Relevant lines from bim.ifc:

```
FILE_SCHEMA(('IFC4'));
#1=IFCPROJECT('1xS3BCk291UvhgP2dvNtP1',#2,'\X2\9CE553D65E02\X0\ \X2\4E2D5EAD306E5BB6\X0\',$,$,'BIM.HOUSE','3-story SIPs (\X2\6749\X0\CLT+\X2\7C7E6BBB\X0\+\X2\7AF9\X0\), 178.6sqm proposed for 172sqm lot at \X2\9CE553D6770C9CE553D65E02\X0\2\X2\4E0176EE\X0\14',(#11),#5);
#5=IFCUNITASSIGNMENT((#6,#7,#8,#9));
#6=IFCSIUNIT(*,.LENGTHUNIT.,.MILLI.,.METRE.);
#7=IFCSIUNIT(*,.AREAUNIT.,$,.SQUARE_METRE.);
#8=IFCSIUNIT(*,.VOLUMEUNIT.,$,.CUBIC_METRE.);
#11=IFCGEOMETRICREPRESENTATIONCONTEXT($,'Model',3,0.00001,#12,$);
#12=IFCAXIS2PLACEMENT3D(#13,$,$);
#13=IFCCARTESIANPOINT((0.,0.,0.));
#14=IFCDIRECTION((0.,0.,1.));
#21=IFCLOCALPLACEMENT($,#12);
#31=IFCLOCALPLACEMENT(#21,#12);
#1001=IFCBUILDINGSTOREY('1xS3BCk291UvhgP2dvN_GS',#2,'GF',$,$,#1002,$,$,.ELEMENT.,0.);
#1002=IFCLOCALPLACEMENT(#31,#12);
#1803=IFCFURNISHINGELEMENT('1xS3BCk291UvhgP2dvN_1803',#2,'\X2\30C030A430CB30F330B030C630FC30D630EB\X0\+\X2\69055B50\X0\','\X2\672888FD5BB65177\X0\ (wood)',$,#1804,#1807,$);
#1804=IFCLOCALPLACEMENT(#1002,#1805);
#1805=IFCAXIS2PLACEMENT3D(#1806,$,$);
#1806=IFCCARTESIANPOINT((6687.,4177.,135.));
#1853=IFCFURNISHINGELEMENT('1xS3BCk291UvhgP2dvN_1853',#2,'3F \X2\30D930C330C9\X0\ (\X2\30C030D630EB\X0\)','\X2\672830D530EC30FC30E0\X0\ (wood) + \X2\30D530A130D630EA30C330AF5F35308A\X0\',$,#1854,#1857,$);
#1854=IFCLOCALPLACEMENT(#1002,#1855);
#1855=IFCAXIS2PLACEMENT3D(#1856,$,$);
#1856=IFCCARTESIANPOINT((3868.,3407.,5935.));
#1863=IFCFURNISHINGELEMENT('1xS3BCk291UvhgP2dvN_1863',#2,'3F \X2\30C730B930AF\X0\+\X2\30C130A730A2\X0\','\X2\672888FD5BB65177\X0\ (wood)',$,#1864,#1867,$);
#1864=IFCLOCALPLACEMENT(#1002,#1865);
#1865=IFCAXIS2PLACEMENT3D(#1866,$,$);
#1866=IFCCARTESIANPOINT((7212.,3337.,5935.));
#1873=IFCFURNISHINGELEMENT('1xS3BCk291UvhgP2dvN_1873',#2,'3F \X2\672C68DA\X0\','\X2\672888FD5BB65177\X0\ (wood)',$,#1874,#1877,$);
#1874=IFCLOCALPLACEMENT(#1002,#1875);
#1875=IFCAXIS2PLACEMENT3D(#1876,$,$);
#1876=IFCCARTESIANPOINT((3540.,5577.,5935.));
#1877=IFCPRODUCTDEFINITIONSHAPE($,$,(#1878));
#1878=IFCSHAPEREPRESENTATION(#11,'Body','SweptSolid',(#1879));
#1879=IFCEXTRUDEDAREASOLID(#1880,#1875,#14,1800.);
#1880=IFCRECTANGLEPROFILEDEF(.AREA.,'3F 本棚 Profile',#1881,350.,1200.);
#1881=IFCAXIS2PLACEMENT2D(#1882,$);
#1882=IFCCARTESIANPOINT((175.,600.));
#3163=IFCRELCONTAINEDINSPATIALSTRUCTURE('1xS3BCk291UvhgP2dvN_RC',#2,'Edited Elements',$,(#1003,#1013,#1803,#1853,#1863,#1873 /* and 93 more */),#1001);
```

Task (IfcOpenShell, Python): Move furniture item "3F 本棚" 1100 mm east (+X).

```python
import ifcopenshell
import ifcopenshell.api.geometry
import ifcopenshell.util.placement
import ifcopenshell.util.unit

model = ifcopenshell.open("bim.ifc")
unit_scale = ifcopenshell.util.unit.calculate_unit_scale(model)

item = model.by_guid("1xS3BCk291UvhgP2dvN_1873")
matrix = ifcopenshell.util.placement.get_local_placement(item.ObjectPlacement)
matrix[0, 3] += 1.1 / unit_scale
ifcopenshell.api.geometry.edit_object_placement(model, product=item, matrix=matrix, is_si=False)

print(ifcopenshell.util.placement.get_local_placement(item.ObjectPlacement).round(3) + 0.0)

model.write("bim_rev.ifc")
```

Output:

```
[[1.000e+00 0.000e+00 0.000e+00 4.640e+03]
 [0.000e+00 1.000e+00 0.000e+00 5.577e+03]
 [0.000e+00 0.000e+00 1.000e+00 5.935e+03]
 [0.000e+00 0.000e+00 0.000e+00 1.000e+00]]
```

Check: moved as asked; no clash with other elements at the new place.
